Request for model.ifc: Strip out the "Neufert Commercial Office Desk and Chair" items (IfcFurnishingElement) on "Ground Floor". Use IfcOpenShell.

First a look at what the model holds.

```python
import ifcopenshell
import ifcopenshell.util.element

model = ifcopenshell.open("model.ifc")
print(model.schema)
storey = next(s for s in model.by_type("IfcBuildingStorey") if s.Name == "Ground Floor")
furniture = [e for e in ifcopenshell.util.element.get_decomposition(storey) if e.is_a("IfcFurnishingElement")]
seen = {}
for e in furniture:
    element_type = ifcopenshell.util.element.get_type(e)
    name = element_type.Name if element_type not in (None, e) else None
    seen[name] = seen.get(name, 0) + 1
for name, count in sorted(seen.items(), key=str):
    print(count, "x", name)
```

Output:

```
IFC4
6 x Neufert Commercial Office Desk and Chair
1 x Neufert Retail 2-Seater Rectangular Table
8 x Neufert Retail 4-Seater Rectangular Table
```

```python
import ifcopenshell
import ifcopenshell.api.root
import ifcopenshell.util.element

model = ifcopenshell.open("model.ifc")

storey = next(s for s in model.by_type("IfcBuildingStorey") if s.Name == "Ground Floor")
furniture = [e for e in ifcopenshell.util.element.get_decomposition(storey) if e.is_a("IfcFurnishingElement")]
targets = [e for e in furniture if (t := ifcopenshell.util.element.get_type(e)) not in (None, e) and t.Name == "Neufert Commercial Office Desk and Chair"]

for e in targets:
    ifcopenshell.api.root.remove_product(model, product=e)
print(len(targets), "removed")

model.write("model_rev.ifc")
```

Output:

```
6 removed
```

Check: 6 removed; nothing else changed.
